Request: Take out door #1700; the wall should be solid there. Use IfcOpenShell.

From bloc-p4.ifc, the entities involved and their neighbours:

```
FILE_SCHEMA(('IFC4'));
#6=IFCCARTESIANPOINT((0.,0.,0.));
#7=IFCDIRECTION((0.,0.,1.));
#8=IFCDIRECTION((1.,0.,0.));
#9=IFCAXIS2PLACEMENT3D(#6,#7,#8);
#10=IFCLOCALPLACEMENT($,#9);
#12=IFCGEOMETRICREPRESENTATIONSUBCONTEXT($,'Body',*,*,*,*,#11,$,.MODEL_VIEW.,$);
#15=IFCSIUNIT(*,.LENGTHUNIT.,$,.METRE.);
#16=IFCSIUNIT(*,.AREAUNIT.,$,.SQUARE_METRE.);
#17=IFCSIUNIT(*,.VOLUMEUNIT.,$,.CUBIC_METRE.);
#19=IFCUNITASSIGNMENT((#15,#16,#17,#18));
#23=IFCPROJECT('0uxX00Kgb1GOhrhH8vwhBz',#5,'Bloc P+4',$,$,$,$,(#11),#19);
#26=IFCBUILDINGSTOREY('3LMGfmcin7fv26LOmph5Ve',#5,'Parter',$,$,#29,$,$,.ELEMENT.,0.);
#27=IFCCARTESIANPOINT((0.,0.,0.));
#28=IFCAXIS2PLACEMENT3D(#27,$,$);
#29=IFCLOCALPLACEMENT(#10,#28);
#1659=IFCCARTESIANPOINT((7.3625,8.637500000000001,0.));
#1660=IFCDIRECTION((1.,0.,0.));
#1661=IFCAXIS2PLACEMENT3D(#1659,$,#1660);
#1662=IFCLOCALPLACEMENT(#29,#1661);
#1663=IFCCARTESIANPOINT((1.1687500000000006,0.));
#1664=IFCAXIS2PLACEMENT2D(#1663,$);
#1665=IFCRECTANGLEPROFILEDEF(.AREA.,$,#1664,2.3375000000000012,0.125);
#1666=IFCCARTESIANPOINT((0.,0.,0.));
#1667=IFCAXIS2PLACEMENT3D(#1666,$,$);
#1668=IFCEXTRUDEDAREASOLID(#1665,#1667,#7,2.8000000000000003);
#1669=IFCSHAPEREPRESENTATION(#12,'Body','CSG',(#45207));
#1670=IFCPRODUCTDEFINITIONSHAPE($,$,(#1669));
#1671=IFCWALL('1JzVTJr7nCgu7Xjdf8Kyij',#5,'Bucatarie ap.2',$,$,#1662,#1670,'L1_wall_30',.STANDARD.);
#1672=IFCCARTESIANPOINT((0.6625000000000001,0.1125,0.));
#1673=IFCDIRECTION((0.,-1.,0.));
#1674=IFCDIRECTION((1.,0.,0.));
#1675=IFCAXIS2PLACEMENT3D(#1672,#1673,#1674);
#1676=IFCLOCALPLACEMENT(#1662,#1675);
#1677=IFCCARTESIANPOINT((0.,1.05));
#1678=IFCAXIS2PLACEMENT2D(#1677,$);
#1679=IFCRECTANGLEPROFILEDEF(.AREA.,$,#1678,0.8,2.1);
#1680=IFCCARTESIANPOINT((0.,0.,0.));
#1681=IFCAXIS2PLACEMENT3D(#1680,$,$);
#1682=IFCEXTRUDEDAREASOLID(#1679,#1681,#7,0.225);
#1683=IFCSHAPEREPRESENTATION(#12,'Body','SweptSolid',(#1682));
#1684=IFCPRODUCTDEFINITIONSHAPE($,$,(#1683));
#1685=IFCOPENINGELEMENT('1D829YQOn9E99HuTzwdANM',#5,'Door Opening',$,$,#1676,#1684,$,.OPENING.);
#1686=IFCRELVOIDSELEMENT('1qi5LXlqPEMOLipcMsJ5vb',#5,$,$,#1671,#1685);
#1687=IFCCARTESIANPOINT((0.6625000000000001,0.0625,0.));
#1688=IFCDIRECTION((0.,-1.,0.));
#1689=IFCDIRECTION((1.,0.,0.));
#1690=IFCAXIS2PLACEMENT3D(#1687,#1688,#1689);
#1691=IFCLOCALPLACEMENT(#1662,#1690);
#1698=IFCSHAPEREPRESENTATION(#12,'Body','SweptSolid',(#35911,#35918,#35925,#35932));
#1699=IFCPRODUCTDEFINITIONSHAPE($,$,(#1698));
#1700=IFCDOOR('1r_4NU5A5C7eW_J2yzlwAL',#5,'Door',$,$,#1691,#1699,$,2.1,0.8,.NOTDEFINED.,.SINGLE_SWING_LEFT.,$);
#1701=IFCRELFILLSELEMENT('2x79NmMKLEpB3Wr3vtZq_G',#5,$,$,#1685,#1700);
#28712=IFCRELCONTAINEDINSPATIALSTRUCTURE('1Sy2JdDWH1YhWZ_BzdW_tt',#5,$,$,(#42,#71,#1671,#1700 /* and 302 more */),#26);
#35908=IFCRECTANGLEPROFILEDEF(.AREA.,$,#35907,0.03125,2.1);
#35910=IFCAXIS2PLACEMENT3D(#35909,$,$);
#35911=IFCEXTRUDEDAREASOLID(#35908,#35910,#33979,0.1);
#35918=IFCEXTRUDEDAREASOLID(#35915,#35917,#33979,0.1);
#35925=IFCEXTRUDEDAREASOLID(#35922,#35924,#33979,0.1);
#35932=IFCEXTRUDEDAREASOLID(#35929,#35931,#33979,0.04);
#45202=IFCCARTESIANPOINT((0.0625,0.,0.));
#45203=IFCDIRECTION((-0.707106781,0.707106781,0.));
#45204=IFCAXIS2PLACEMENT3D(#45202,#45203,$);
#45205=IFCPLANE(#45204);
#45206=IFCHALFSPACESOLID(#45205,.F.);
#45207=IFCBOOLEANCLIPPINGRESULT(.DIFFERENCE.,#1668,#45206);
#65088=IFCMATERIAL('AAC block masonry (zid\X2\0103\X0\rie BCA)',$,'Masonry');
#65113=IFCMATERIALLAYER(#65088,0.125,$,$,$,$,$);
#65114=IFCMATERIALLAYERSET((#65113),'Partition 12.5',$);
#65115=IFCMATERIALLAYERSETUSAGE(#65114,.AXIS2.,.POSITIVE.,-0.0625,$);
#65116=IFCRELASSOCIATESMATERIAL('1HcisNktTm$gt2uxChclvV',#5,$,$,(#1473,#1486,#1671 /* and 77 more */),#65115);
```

```python
import ifcopenshell
import ifcopenshell.api.feature
import ifcopenshell.api.root
import ifcopenshell.geom
import ifcopenshell.util.shape

model = ifcopenshell.open("bloc-p4.ifc")
settings = ifcopenshell.geom.settings()


def volume(element):
    """Net volume in cubic metres, openings subtracted."""
    shape = ifcopenshell.geom.create_shape(settings, element)
    return ifcopenshell.util.shape.get_volume(shape.geometry)


door = model.by_id(1700)
opening = door.FillsVoids[0].RelatingOpeningElement
wall = opening.VoidsElements[0].RelatingBuildingElement
before = volume(wall)

ifcopenshell.api.root.remove_product(model, product=door)
ifcopenshell.api.feature.remove_feature(model, feature=opening)

after = volume(wall)

print(f"wall volume {before:.3f} -> {after:.3f} m3")

model.write("bloc-p4_edited.ifc")
```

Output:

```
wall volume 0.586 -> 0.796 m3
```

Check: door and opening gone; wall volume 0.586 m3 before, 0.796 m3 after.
